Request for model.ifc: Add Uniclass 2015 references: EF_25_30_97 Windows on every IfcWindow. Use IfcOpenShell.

First a look at what the model holds.

```python
import ifcopenshell

model = ifcopenshell.open("model.ifc")
print(model.schema)
print("classifications:", [c.Name for c in model.by_type("IfcClassification")])
for ifc_class in ("IfcDoor", "IfcRoof", "IfcStair", "IfcWall", "IfcWindow"):
    print(ifc_class, len(model.by_type(ifc_class)))
```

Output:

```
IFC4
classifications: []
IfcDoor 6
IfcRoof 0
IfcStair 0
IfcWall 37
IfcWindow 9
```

```python
import ifcopenshell
import ifcopenshell.api.classification

model = ifcopenshell.open("model.ifc")

system = ifcopenshell.api.classification.add_classification(model, classification="Uniclass 2015")

codes = {
    "IfcWindow": ("EF_25_30_97", "Windows"),
}
for ifc_class, (code, name) in codes.items():
    products = model.by_type(ifc_class)
    ifcopenshell.api.classification.add_reference(
        model, products=products, classification=system, identification=code, name=name
    )
    print(code, len(products))

model.write("model_edited.ifc")
```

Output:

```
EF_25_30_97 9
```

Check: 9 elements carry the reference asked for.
